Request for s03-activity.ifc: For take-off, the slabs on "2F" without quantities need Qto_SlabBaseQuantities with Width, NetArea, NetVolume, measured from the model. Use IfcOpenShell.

First a look at what the model holds.

```python
import ifcopenshell
import ifcopenshell.util.element
import ifcopenshell.util.unit

model = ifcopenshell.open("s03-activity.ifc")
print(model.schema)
for unit_type in ("LENGTHUNIT", "AREAUNIT", "VOLUMEUNIT"):
    print(unit_type, ifcopenshell.util.unit.calculate_unit_scale(model, unit_type))
storey = next(s for s in model.by_type("IfcBuildingStorey") if s.Name == "2F")
slabs = [e for e in ifcopenshell.util.element.get_decomposition(storey) if e.is_a("IfcSlab")]
for e in sorted(slabs, key=lambda e: e.id()):
    print(e.id(), e.is_a(), e.Name, list(ifcopenshell.util.element.get_psets(e, qtos_only=True)), sep=" | ")
```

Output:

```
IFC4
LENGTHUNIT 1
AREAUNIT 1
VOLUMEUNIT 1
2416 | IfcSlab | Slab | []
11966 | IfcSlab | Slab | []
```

```python
import ifcopenshell
import ifcopenshell.api.pset
import ifcopenshell.geom
import ifcopenshell.util.element
import ifcopenshell.util.shape
import ifcopenshell.util.unit

model = ifcopenshell.open("s03-activity.ifc")
unit_scale = ifcopenshell.util.unit.calculate_unit_scale(model)
area_scale = ifcopenshell.util.unit.calculate_unit_scale(model, "AREAUNIT")
volume_scale = ifcopenshell.util.unit.calculate_unit_scale(model, "VOLUMEUNIT")
settings = ifcopenshell.geom.settings()

storey = next(s for s in model.by_type("IfcBuildingStorey") if s.Name == "2F")
slabs = [e for e in ifcopenshell.util.element.get_decomposition(storey) if e.is_a("IfcSlab")]

for e in sorted(slabs, key=lambda e: e.id()):
    if ifcopenshell.util.element.get_psets(e, qtos_only=True, should_inherit=False):
        continue
    # Geometry comes back in metres, in the element's own axes.
    shape = ifcopenshell.geom.create_shape(settings, e)
    values = {
        "Width": ifcopenshell.util.shape.get_z(shape.geometry) / unit_scale,
        "NetArea": ifcopenshell.util.shape.get_footprint_area(shape.geometry) / area_scale,
        "NetVolume": ifcopenshell.util.shape.get_volume(shape.geometry) / volume_scale,
    }
    qto = ifcopenshell.api.pset.add_qto(model, product=e, name="Qto_SlabBaseQuantities")
    ifcopenshell.api.pset.edit_qto(model, qto=qto, properties=values)
    print(e.id(), {k: round(v, 3) for k, v in values.items()})

model.write("s03-activity-out.ifc")
```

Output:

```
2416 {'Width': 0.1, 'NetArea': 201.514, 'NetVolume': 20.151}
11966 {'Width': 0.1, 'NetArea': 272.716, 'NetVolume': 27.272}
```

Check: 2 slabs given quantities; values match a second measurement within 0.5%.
